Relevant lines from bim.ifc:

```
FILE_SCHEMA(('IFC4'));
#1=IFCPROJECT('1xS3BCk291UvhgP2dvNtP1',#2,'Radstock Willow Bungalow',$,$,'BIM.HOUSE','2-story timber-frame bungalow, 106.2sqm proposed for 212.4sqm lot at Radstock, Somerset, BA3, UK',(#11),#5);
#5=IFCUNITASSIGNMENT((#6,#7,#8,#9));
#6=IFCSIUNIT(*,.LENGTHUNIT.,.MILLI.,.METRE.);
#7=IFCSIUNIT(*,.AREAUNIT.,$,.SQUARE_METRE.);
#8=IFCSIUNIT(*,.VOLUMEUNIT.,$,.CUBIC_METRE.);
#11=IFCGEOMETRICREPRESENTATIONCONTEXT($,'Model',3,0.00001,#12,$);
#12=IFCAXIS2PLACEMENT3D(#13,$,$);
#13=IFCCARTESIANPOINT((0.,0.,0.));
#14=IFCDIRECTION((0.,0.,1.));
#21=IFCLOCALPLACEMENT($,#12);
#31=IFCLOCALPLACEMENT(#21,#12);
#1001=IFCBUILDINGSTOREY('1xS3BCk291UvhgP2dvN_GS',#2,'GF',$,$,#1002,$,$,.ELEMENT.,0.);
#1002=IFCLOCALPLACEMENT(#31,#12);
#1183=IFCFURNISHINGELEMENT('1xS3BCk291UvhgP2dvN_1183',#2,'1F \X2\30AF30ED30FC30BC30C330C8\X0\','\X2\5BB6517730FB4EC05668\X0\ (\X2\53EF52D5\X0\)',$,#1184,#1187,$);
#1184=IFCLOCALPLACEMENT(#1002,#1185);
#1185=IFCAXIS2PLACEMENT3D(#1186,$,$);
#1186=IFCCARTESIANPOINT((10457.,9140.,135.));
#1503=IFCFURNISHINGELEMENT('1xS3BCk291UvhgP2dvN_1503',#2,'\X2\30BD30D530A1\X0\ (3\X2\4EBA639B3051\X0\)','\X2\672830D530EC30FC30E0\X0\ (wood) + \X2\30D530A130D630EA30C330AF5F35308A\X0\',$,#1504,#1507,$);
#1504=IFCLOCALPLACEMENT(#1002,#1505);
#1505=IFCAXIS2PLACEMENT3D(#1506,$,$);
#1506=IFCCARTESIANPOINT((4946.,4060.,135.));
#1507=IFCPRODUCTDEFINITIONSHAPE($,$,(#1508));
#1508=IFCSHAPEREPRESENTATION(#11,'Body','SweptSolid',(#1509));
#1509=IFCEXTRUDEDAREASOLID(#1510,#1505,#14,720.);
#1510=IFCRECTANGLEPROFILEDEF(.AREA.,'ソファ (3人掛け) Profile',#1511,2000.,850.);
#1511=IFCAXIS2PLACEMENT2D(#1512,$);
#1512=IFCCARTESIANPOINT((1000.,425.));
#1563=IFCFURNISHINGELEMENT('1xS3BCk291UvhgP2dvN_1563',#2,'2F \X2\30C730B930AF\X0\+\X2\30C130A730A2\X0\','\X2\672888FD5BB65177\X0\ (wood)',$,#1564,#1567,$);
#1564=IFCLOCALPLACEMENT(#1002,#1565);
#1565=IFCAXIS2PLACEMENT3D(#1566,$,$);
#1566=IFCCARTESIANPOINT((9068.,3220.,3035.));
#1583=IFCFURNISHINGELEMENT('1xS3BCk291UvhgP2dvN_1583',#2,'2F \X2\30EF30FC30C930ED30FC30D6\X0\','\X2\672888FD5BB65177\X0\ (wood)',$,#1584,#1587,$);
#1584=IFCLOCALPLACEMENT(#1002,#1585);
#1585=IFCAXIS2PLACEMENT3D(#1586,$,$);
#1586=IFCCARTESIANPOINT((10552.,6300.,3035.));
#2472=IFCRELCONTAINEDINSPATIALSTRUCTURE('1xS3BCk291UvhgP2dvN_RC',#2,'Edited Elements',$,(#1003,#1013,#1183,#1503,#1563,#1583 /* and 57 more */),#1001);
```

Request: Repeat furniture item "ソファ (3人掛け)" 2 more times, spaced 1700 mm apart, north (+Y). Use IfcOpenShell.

```python
import numpy as np
import ifcopenshell
import ifcopenshell.api.geometry
import ifcopenshell.api.root
import ifcopenshell.util.element
import ifcopenshell.util.placement

model = ifcopenshell.open("bim.ifc")


def reuse_history(source, copy):
    """copy_class also copies each property set's owner history, people and application; keep the originals."""
    for rel in copy.IsDefinedBy:
        if rel.is_a("IfcRelDefinesByProperties") and (history := rel.RelatingPropertyDefinition.OwnerHistory):
            rel.RelatingPropertyDefinition.OwnerHistory = source.OwnerHistory
            ifcopenshell.util.element.remove_deep2(model, history)


source = model.by_guid("1xS3BCk291UvhgP2dvN_1503")
base = ifcopenshell.util.placement.get_local_placement(source.ObjectPlacement)
step = np.array([0.0, 1.0, 0.0]) * 1700.0

for i in range(1, 3):
    copy = ifcopenshell.api.root.copy_class(model, product=source)
    copy.Representation = ifcopenshell.util.element.copy_deep(
        model, source.Representation, exclude=["IfcGeometricRepresentationContext", "IfcRepresentationMap"]
    )
    reuse_history(source, copy)
    matrix = base.copy()
    matrix[:3, 3] += i * step
    print("added at", matrix[:3, 3].round(3) + 0.0)
    ifcopenshell.api.geometry.edit_object_placement(model, product=copy, matrix=matrix, is_si=False)

model.write("bim_edited.ifc")
```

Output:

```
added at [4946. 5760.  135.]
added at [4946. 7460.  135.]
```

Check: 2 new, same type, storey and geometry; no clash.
